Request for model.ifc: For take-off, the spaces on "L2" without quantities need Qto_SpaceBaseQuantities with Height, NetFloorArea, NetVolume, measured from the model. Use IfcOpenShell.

First a look at what the model holds.

```python
import ifcopenshell
import ifcopenshell.util.element
import ifcopenshell.util.unit

model = ifcopenshell.open("model.ifc")
print(model.schema)
for unit_type in ("LENGTHUNIT", "AREAUNIT", "VOLUMEUNIT"):
    print(unit_type, ifcopenshell.util.unit.calculate_unit_scale(model, unit_type))
storey = next(s for s in model.by_type("IfcBuildingStorey") if s.Name == "L2")
spaces = [e for e in ifcopenshell.util.element.get_decomposition(storey) if e.is_a("IfcSpace")]
for e in sorted(spaces, key=lambda e: e.id()):
    print(e.id(), e.is_a(), e.Name, list(ifcopenshell.util.element.get_psets(e, qtos_only=True)), sep=" | ")
```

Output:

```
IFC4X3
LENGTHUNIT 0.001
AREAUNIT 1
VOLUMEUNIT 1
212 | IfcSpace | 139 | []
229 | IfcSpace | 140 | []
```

```python
import ifcopenshell
import ifcopenshell.api.pset
import ifcopenshell.geom
import ifcopenshell.util.element
import ifcopenshell.util.shape
import ifcopenshell.util.unit

model = ifcopenshell.open("model.ifc")
unit_scale = ifcopenshell.util.unit.calculate_unit_scale(model)
area_scale = ifcopenshell.util.unit.calculate_unit_scale(model, "AREAUNIT")
volume_scale = ifcopenshell.util.unit.calculate_unit_scale(model, "VOLUMEUNIT")
settings = ifcopenshell.geom.settings()

storey = next(s for s in model.by_type("IfcBuildingStorey") if s.Name == "L2")
spaces = [e for e in ifcopenshell.util.element.get_decomposition(storey) if e.is_a("IfcSpace")]

for e in sorted(spaces, key=lambda e: e.id()):
    if ifcopenshell.util.element.get_psets(e, qtos_only=True, should_inherit=False):
        continue
    # Geometry comes back in metres, in the element's own axes.
    shape = ifcopenshell.geom.create_shape(settings, e)
    values = {
        "Height": ifcopenshell.util.shape.get_z(shape.geometry) / unit_scale,
        "NetFloorArea": ifcopenshell.util.shape.get_footprint_area(shape.geometry) / area_scale,
        "NetVolume": ifcopenshell.util.shape.get_volume(shape.geometry) / volume_scale,
    }
    qto = ifcopenshell.api.pset.add_qto(model, product=e, name="Qto_SpaceBaseQuantities")
    ifcopenshell.api.pset.edit_qto(model, qto=qto, properties=values)
    print(e.id(), {k: round(v, 3) for k, v in values.items()})

model.write("model-out.ifc")
```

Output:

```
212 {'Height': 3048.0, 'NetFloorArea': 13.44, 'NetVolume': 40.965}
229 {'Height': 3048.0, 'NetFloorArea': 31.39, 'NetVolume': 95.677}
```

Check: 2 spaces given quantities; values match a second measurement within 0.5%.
